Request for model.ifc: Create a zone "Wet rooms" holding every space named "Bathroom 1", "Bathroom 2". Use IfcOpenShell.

First a look at what the model holds.

```python
import ifcopenshell

model = ifcopenshell.open("model.ifc")
print(model.schema)
seen = {}
for space in model.by_type("IfcSpace"):
    seen[space.LongName] = seen.get(space.LongName, 0) + 1
for name, count in sorted(seen.items(), key=str):
    print(count, "x", name)
print("zones:", [z.Name for z in model.by_type("IfcZone")][:20])
```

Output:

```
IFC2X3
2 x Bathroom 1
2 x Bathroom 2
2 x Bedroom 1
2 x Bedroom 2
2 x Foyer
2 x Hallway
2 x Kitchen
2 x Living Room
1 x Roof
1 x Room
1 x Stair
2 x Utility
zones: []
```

```python
import ifcopenshell
import ifcopenshell.api.group
import ifcopenshell.api.root

model = ifcopenshell.open("model.ifc")

names = {"Bathroom 1", "Bathroom 2"}
spaces = [s for s in model.by_type("IfcSpace") if s.LongName in names]

zone = ifcopenshell.api.root.create_entity(model, ifc_class="IfcZone", name="Wet rooms")
ifcopenshell.api.group.assign_group(model, products=spaces, group=zone)
print(len(spaces), "spaces in", zone.Name)

model.write("model_edited.ifc")
```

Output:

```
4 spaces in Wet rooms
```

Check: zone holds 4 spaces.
